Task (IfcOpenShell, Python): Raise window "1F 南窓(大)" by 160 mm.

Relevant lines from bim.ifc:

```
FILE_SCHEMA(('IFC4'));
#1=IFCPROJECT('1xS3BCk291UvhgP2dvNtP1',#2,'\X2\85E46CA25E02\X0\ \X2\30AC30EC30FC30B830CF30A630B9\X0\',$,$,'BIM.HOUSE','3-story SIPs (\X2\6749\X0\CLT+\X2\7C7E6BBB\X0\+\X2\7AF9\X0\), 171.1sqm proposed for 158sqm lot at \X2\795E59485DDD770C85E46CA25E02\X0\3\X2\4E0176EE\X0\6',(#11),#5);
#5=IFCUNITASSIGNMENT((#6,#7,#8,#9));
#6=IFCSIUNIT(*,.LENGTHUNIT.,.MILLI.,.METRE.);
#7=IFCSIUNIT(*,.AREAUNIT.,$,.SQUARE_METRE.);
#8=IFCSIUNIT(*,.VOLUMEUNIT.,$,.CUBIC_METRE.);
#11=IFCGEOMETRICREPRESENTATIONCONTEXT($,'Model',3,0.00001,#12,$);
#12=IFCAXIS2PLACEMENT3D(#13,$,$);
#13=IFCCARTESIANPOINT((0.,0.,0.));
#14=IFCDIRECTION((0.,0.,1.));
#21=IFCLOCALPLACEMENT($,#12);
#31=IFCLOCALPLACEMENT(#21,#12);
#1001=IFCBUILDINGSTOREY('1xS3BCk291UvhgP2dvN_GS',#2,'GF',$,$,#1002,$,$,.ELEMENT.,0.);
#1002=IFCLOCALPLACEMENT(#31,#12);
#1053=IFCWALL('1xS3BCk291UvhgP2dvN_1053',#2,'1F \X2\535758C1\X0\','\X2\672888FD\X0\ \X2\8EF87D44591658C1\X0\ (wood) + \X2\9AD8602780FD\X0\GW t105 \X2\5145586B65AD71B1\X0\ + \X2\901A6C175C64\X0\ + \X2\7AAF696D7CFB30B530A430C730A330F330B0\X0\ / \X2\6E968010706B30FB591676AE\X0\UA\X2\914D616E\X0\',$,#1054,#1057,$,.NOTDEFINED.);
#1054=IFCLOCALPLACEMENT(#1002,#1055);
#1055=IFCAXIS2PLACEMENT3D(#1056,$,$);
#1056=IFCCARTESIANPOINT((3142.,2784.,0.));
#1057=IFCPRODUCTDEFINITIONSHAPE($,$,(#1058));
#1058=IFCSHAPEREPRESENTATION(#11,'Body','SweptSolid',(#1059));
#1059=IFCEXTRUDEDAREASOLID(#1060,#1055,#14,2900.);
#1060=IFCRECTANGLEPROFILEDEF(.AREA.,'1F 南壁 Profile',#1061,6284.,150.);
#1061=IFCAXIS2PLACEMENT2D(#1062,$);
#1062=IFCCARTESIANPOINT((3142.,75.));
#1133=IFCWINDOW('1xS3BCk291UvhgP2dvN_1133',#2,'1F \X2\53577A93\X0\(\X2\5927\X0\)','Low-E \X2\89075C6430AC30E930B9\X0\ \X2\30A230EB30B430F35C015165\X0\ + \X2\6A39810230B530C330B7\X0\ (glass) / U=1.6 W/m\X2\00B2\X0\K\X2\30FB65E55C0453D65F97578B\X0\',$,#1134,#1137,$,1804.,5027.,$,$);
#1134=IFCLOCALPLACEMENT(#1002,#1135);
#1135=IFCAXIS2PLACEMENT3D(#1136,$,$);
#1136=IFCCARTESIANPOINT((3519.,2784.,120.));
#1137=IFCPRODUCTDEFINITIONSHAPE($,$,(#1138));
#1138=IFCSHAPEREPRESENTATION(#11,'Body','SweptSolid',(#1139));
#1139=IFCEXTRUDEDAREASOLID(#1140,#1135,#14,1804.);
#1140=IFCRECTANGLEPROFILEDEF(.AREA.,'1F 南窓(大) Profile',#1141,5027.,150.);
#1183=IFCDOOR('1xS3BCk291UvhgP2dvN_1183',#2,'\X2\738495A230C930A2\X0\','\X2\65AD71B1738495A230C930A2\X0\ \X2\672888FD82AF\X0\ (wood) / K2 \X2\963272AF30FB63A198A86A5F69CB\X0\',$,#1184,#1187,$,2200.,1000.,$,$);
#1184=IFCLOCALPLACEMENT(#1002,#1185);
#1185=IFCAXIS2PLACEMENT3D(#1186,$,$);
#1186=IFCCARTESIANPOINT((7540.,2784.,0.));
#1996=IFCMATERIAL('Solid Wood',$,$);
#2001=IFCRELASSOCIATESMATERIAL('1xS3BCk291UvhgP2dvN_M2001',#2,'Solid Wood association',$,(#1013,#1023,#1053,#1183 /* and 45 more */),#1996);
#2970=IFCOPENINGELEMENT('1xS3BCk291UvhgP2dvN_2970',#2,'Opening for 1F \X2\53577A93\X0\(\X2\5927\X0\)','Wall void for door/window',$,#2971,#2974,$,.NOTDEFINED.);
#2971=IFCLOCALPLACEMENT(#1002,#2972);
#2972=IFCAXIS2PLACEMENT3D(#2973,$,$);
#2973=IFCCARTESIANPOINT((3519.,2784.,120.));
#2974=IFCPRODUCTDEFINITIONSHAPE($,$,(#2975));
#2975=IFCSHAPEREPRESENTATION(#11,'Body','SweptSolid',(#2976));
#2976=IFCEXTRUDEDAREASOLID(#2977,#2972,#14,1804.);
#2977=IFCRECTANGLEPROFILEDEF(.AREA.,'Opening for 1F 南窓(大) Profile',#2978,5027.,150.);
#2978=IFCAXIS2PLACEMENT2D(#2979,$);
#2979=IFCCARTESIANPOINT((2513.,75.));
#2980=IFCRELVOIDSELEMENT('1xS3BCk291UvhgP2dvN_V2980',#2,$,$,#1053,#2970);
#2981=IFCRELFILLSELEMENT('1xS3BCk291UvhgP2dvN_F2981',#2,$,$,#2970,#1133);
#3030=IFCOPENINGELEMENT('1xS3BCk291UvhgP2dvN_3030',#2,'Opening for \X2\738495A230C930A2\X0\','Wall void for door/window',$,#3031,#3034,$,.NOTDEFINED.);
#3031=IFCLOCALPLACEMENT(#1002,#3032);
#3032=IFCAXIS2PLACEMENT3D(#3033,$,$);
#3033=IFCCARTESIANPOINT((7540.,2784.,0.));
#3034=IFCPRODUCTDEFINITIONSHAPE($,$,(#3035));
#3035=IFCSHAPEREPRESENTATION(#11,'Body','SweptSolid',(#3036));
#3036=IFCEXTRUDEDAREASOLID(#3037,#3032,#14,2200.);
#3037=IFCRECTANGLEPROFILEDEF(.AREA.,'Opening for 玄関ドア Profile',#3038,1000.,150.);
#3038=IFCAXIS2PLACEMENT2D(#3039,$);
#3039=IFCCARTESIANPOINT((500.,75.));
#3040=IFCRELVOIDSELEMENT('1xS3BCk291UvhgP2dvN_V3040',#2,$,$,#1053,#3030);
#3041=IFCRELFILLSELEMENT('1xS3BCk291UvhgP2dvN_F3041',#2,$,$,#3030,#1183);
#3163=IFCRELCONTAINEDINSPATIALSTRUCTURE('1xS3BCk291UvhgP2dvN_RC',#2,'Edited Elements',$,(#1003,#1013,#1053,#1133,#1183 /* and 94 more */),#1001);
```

```python
import numpy as np
import ifcopenshell
import ifcopenshell.api.geometry
import ifcopenshell.util.placement
import ifcopenshell.util.unit

model = ifcopenshell.open("bim.ifc")
unit_scale = ifcopenshell.util.unit.calculate_unit_scale(model)

window = model.by_guid("1xS3BCk291UvhgP2dvN_1133")
opening = window.FillsVoids[0].RelatingOpeningElement
dz = 0.16 / unit_scale

shift = np.array([0.0, 0.0, dz])
# The window is not placed relative to its opening, so move both.
for product in (opening, window):
    matrix = ifcopenshell.util.placement.get_local_placement(product.ObjectPlacement)
    matrix[:3, 3] += shift
    ifcopenshell.api.geometry.edit_object_placement(model, product=product, matrix=matrix, is_si=False)

print(f"moved by {dz * unit_scale:+.3f} m")

model.write("bim-out.ifc")
```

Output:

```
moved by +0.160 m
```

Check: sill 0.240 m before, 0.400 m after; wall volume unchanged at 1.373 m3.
